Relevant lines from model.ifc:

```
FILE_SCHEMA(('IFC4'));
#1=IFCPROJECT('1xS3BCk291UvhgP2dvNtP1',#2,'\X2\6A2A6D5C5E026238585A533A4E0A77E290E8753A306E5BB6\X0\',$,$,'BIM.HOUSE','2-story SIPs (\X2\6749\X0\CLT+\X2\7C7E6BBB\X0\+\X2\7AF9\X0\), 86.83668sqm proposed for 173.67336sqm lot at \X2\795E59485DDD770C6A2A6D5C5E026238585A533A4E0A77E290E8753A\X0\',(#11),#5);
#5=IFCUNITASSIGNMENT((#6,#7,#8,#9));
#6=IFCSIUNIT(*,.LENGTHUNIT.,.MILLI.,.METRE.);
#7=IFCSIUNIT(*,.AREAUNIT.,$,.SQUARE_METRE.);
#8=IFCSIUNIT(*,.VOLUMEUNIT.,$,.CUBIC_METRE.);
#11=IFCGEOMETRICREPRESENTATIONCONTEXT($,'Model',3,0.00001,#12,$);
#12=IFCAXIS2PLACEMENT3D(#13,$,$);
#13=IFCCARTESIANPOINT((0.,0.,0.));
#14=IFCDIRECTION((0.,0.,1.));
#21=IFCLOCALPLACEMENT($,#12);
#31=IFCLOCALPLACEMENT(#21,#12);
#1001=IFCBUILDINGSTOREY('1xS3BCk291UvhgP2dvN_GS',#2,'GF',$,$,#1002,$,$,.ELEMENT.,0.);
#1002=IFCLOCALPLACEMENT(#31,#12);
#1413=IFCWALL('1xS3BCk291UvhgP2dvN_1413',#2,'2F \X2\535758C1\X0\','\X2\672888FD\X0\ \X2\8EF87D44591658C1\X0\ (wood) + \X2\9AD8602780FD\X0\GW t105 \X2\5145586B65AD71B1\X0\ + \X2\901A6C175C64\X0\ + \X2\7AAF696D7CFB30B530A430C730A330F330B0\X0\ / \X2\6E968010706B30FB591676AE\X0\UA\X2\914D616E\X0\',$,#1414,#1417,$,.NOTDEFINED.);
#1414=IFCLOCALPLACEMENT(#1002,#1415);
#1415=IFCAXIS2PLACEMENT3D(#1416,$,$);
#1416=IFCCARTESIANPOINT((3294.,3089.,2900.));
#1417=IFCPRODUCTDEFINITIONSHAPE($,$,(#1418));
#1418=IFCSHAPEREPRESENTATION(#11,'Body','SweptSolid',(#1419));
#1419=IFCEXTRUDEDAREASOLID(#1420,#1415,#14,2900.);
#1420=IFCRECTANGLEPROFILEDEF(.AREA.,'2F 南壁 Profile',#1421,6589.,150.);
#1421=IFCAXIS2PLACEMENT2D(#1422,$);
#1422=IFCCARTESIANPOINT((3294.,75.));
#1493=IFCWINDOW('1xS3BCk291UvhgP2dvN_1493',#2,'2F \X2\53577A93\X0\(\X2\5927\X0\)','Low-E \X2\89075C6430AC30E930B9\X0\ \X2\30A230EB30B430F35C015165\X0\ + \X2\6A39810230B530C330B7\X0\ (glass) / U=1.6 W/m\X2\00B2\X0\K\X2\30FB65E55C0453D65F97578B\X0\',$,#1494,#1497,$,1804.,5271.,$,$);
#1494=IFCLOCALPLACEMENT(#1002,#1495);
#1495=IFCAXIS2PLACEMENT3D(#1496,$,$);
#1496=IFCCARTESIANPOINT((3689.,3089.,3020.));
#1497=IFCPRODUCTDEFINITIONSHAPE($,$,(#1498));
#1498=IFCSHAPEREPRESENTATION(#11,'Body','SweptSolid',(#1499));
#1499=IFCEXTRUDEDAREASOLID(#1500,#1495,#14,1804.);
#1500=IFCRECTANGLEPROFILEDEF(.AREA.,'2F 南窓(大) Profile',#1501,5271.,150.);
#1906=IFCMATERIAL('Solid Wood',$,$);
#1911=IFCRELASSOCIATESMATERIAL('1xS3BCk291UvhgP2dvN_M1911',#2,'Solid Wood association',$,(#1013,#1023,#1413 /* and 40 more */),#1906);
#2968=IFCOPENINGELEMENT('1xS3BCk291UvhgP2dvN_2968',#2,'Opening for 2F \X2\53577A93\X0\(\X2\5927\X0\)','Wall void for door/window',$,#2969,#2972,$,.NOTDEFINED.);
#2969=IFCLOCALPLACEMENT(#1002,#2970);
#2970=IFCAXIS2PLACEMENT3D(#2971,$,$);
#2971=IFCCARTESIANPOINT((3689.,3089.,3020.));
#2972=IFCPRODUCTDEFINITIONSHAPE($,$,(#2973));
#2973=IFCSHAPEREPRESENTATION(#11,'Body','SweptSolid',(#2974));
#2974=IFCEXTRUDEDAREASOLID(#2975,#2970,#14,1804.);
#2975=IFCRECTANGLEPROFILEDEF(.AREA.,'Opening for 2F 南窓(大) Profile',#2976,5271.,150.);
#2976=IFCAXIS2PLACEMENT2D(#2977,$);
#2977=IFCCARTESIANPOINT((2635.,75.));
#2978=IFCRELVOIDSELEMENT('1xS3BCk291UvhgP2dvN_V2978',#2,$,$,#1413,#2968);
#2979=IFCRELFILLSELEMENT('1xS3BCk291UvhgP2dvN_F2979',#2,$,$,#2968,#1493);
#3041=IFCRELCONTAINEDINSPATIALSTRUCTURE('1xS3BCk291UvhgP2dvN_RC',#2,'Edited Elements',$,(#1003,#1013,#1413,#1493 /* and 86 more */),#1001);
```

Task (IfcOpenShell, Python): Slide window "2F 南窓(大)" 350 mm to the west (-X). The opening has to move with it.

```python
import ifcopenshell
import ifcopenshell.api.geometry
import ifcopenshell.util.placement
import ifcopenshell.util.unit

model = ifcopenshell.open("model.ifc")
unit_scale = ifcopenshell.util.unit.calculate_unit_scale(model)

window = model.by_guid("1xS3BCk291UvhgP2dvN_1493")
opening = window.FillsVoids[0].RelatingOpeningElement
wall = opening.VoidsElements[0].RelatingBuildingElement

wall_matrix = ifcopenshell.util.placement.get_local_placement(wall.ObjectPlacement)
shift = wall_matrix[:3, 0] * -0.35 / unit_scale
before = ifcopenshell.util.placement.get_local_placement(window.ObjectPlacement)[:3, 3].copy()

# The window is not placed relative to its opening, so move both.
for product in (opening, window):
    matrix = ifcopenshell.util.placement.get_local_placement(product.ObjectPlacement)
    matrix[:3, 3] += shift
    ifcopenshell.api.geometry.edit_object_placement(model, product=product, matrix=matrix, is_si=False)

after = ifcopenshell.util.placement.get_local_placement(window.ObjectPlacement)[:3, 3]
print("window moved by", (after - before).round(3) + 0.0)

model.write("model_v2.ifc")
```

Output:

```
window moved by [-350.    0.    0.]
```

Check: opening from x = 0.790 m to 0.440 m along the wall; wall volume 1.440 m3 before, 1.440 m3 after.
